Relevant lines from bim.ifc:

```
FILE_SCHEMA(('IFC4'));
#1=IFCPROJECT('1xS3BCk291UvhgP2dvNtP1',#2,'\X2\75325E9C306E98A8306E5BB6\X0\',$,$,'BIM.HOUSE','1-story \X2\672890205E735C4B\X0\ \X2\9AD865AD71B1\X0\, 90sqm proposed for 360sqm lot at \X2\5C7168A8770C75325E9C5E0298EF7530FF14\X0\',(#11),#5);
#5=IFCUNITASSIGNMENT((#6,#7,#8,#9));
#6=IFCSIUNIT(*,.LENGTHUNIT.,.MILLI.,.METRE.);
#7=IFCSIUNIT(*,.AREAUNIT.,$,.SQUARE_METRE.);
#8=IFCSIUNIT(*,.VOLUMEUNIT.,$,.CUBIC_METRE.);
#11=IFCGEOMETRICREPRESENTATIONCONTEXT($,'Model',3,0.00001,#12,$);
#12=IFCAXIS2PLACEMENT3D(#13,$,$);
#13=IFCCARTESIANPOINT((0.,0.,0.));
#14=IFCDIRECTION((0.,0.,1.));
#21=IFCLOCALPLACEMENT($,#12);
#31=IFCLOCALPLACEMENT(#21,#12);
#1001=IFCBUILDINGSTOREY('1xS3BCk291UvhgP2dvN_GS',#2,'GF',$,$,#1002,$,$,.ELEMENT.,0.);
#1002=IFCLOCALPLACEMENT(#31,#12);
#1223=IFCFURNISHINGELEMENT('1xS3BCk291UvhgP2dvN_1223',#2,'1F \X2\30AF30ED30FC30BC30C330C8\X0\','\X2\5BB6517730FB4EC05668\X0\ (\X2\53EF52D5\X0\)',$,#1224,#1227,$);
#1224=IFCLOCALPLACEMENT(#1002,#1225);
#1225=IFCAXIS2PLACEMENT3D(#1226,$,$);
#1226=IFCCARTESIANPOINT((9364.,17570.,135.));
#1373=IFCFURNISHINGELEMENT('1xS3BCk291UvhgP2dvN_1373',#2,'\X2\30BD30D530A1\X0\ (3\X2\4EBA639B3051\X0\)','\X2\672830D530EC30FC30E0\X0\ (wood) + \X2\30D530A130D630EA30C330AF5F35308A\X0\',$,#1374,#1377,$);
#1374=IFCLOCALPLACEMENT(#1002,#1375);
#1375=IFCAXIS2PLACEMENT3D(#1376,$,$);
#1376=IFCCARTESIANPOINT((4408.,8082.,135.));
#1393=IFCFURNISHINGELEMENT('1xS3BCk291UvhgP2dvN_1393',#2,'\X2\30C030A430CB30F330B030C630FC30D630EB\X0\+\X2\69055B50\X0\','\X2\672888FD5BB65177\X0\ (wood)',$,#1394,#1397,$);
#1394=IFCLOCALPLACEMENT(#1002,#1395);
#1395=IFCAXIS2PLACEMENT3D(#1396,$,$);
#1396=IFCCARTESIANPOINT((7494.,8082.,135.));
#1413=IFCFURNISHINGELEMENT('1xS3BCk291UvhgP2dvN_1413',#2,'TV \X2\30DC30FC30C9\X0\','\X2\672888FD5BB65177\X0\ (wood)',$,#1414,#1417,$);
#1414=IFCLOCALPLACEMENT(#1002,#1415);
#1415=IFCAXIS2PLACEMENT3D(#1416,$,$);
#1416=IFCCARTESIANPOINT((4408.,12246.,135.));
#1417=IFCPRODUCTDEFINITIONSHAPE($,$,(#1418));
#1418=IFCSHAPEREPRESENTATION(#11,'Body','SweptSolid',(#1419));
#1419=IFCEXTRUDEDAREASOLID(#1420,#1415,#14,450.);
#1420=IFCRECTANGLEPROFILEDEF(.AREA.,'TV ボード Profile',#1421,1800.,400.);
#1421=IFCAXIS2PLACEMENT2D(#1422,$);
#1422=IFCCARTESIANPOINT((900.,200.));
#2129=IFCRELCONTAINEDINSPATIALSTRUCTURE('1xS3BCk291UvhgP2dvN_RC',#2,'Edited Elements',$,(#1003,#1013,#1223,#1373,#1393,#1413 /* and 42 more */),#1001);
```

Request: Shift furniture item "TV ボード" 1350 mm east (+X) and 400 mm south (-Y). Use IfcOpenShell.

```python
import ifcopenshell
import ifcopenshell.api.geometry
import ifcopenshell.util.placement

model = ifcopenshell.open("bim.ifc")

item = model.by_id(1413)
matrix = ifcopenshell.util.placement.get_local_placement(item.ObjectPlacement)
matrix[0, 3] += 1350.0
matrix[1, 3] -= 400.0
ifcopenshell.api.geometry.edit_object_placement(model, product=item, matrix=matrix, is_si=False)

print(ifcopenshell.util.placement.get_local_placement(item.ObjectPlacement).round(3) + 0.0)

model.write("bim_edited.ifc")
```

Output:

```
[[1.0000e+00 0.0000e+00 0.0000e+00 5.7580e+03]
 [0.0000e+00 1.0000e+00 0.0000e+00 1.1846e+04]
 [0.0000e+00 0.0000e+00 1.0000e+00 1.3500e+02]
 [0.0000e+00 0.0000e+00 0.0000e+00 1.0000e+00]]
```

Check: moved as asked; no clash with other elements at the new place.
